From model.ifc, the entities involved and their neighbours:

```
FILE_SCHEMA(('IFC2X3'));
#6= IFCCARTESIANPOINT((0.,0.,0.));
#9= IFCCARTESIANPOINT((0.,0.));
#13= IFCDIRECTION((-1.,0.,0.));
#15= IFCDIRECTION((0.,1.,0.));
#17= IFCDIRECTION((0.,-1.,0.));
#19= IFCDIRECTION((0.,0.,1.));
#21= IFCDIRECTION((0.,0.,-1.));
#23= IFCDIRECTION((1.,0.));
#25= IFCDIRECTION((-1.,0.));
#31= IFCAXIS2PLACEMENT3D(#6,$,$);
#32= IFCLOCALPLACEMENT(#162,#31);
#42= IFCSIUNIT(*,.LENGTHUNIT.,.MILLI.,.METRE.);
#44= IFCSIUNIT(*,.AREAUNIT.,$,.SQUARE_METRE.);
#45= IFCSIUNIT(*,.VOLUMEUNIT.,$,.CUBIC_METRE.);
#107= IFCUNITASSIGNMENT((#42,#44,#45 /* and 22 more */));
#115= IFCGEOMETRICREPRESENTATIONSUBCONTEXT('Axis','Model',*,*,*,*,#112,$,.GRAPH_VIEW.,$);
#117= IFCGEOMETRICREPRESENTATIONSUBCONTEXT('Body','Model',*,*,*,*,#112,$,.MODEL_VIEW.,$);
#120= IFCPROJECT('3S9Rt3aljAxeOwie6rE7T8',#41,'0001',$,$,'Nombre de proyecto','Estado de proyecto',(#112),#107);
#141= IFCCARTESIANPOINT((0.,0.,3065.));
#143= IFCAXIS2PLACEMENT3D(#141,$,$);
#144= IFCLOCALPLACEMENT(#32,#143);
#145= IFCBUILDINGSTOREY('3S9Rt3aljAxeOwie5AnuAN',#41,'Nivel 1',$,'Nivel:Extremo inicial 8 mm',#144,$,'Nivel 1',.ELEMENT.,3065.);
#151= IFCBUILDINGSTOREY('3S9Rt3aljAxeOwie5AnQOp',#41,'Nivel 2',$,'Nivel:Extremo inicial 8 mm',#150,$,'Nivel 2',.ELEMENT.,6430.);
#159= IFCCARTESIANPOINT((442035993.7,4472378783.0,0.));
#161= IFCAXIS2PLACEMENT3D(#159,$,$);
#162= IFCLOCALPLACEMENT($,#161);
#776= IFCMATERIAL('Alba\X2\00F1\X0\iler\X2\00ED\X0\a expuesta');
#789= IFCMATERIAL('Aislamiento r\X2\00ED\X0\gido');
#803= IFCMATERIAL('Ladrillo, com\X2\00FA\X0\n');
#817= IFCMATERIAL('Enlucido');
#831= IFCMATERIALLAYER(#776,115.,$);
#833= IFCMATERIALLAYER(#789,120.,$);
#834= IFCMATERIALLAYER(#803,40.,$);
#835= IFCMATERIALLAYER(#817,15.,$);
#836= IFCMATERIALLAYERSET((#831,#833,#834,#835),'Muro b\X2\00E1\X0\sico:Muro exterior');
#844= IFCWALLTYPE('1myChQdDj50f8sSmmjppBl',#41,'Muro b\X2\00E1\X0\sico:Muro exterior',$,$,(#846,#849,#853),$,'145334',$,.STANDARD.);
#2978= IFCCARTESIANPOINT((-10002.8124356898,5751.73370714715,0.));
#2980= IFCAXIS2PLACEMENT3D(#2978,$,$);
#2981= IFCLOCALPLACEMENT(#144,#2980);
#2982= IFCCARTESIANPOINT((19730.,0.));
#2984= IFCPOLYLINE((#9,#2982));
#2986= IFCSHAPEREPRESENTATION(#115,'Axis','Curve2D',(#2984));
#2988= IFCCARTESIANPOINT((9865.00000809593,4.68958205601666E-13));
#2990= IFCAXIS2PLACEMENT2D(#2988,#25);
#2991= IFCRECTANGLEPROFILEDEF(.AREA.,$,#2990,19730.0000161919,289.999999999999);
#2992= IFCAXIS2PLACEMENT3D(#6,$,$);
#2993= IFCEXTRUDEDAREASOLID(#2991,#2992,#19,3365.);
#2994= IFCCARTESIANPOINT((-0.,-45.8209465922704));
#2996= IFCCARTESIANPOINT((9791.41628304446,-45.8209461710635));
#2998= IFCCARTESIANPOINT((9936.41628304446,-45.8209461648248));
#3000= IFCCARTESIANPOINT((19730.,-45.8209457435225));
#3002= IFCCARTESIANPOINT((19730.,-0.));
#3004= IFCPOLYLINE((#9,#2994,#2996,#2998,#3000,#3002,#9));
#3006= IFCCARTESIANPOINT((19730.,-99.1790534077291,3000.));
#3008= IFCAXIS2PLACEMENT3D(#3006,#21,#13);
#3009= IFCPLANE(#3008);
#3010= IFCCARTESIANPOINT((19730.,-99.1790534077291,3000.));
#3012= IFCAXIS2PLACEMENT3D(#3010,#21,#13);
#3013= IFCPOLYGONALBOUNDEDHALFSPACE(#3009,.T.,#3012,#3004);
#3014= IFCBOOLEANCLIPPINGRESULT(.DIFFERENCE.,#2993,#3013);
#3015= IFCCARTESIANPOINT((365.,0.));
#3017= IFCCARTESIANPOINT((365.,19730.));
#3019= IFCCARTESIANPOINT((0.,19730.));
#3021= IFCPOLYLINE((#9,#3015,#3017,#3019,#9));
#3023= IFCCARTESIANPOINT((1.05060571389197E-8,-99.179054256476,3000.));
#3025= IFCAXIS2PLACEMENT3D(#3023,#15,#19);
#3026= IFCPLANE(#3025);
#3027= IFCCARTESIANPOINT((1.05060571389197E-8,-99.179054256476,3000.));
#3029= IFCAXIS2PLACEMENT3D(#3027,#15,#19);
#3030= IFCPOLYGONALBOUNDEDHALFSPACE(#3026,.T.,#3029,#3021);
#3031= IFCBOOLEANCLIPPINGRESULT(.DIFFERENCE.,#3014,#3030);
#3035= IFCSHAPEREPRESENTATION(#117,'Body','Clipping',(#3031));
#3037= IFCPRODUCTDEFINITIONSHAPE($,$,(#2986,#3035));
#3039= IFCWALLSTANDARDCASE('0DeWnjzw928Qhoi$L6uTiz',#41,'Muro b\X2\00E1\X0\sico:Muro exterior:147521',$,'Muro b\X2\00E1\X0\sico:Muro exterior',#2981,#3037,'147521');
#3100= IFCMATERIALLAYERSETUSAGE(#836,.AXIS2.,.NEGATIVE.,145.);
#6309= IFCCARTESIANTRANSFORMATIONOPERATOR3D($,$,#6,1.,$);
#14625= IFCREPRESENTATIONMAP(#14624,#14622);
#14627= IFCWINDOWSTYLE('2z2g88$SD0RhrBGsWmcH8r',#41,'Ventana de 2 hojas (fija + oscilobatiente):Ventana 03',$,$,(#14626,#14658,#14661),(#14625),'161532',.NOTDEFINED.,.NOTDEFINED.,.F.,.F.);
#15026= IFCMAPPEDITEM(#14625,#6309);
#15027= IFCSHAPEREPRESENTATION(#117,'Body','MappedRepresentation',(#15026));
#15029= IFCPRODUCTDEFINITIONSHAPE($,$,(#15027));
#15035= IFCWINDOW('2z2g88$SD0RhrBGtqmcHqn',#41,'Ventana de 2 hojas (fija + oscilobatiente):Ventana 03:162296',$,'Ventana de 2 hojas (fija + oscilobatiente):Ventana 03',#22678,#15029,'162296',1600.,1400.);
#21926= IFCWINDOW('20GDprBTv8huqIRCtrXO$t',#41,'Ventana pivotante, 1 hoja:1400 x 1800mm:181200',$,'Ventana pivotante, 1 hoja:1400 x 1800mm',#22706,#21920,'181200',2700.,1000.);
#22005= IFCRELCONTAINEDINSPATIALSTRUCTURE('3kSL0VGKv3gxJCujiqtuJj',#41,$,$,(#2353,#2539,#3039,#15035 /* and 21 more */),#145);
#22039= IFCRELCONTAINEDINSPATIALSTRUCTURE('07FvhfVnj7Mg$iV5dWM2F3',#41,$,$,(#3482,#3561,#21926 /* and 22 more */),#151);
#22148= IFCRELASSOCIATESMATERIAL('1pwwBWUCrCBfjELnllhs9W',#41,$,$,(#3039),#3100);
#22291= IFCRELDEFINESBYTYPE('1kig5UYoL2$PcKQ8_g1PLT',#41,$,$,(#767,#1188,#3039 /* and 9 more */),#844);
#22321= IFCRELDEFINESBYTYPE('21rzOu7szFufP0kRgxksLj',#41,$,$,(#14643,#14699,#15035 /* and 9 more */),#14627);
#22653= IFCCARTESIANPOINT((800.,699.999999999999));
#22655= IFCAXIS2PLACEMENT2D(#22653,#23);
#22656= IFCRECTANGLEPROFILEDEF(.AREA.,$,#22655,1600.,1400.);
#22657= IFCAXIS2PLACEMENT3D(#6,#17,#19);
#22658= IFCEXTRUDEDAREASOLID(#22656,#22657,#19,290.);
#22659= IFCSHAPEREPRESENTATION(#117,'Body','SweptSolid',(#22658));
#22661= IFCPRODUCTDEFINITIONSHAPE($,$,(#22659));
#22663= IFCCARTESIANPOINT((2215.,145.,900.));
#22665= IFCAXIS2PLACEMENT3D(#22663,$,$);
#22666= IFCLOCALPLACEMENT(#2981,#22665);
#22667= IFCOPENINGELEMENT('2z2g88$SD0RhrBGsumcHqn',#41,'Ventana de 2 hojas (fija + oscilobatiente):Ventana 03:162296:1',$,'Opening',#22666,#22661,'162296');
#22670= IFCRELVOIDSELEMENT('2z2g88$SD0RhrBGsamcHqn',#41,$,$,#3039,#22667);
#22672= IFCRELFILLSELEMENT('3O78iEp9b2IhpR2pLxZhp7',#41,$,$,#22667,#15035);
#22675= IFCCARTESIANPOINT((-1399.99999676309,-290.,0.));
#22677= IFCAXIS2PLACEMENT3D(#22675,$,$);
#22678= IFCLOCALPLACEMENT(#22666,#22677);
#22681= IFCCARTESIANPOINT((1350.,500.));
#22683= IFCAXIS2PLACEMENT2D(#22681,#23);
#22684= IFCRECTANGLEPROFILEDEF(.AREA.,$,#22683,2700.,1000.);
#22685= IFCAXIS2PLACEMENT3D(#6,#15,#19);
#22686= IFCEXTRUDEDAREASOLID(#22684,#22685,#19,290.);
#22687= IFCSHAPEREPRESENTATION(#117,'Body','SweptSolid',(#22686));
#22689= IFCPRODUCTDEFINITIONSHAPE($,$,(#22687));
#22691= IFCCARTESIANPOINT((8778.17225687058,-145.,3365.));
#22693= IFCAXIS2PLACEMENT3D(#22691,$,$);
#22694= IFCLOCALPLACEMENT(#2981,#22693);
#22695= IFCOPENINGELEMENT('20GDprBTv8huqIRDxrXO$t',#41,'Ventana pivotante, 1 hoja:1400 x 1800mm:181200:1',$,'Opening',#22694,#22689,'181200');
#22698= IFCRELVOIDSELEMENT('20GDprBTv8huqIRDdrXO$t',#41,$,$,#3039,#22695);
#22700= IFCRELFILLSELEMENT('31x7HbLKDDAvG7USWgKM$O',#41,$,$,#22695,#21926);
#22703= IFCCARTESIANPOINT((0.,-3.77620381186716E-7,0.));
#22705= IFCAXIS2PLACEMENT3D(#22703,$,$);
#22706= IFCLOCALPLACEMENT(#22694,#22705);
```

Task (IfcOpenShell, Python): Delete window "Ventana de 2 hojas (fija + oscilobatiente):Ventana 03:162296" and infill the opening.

```python
import ifcopenshell
import ifcopenshell.api.feature
import ifcopenshell.api.root
import ifcopenshell.geom
import ifcopenshell.util.shape

model = ifcopenshell.open("model.ifc")
settings = ifcopenshell.geom.settings()


def volume(element):
    """Net volume in cubic metres, openings subtracted."""
    shape = ifcopenshell.geom.create_shape(settings, element)
    return ifcopenshell.util.shape.get_volume(shape.geometry)


window = model.by_guid("2z2g88$SD0RhrBGtqmcHqn")
opening = window.FillsVoids[0].RelatingOpeningElement
wall = opening.VoidsElements[0].RelatingBuildingElement
before = volume(wall)

ifcopenshell.api.root.remove_product(model, product=window)
ifcopenshell.api.feature.remove_feature(model, feature=opening)

after = volume(wall)

print(f"wall volume {before:.3f} -> {after:.3f} m3")

model.write("model_updated.ifc")
```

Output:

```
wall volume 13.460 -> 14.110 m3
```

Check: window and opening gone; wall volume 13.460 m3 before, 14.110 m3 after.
